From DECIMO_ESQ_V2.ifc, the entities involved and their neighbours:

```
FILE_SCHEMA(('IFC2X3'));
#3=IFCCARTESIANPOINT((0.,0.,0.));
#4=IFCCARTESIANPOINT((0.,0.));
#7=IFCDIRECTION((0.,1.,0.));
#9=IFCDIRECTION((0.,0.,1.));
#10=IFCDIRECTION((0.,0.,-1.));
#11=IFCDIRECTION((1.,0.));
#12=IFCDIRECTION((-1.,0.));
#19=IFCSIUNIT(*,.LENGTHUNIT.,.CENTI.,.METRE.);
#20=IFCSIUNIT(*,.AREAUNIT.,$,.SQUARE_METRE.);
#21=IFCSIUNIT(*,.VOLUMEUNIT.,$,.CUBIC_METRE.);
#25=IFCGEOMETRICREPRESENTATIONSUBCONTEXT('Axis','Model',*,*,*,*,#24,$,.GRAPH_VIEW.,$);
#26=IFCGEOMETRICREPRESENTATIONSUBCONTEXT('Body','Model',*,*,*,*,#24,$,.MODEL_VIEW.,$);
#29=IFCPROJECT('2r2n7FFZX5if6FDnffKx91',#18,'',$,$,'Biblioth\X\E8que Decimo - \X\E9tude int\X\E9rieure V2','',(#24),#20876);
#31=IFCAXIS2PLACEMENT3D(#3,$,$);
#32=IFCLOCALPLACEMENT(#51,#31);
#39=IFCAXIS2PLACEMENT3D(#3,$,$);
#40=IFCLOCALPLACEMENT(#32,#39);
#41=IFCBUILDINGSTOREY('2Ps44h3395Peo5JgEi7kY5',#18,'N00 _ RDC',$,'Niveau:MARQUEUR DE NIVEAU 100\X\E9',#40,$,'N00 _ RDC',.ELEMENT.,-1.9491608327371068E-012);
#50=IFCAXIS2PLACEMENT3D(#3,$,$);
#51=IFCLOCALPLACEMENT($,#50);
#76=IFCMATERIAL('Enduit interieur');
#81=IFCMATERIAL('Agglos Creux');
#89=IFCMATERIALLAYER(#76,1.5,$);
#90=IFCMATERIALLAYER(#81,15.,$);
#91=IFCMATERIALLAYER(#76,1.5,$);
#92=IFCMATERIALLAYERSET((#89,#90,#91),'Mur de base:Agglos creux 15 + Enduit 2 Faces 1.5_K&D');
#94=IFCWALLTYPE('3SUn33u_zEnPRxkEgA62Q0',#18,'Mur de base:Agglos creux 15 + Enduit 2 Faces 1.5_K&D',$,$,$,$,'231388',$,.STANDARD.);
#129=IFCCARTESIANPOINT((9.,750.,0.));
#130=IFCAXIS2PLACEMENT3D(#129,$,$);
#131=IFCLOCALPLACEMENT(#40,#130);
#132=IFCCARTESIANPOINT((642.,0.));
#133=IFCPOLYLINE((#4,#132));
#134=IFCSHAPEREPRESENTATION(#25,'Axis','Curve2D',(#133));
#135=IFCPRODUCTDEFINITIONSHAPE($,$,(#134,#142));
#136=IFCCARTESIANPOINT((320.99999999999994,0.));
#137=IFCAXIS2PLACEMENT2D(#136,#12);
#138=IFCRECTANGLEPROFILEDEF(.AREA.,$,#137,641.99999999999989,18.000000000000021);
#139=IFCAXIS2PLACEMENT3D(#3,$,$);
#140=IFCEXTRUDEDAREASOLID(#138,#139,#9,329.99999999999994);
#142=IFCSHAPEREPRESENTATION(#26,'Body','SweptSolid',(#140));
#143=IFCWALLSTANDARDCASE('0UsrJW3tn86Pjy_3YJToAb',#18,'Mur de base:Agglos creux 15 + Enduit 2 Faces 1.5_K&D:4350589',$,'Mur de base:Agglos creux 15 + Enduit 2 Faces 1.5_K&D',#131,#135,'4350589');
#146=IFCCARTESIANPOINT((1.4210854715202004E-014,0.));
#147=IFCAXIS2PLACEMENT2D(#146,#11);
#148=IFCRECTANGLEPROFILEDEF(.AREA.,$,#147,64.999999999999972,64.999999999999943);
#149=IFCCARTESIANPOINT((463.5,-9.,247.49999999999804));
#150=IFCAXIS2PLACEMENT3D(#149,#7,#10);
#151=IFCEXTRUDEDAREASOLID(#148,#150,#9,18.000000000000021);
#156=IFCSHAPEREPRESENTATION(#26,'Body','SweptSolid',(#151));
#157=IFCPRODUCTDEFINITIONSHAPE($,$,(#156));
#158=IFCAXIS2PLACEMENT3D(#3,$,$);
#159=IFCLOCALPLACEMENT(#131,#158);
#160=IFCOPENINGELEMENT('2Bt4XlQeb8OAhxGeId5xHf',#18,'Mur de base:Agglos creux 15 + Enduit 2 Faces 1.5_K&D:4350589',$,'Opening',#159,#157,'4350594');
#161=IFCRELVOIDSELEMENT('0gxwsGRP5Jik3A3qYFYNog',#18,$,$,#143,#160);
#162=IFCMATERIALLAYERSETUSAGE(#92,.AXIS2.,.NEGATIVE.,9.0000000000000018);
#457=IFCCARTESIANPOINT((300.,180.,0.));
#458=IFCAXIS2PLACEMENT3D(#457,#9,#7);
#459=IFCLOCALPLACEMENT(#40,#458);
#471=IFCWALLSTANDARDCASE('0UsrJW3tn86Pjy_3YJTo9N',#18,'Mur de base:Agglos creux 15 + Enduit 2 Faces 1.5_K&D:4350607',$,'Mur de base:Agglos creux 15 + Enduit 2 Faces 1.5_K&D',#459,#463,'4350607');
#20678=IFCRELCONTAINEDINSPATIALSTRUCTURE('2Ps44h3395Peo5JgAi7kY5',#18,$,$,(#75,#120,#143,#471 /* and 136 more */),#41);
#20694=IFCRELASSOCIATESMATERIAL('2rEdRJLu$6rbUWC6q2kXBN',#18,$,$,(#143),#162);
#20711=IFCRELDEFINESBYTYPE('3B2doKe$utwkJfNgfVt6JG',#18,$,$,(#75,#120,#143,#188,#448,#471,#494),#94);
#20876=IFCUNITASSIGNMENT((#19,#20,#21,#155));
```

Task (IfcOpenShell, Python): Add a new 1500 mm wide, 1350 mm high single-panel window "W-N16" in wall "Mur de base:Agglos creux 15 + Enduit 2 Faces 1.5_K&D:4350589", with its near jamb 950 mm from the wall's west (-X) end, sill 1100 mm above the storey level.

```python
import numpy as np
import ifcopenshell
import ifcopenshell.api.feature
import ifcopenshell.api.geometry
import ifcopenshell.api.root
import ifcopenshell.api.spatial
import ifcopenshell.api.type
import ifcopenshell.geom
import ifcopenshell.util.element
import ifcopenshell.util.placement
import ifcopenshell.util.representation
import ifcopenshell.util.shape
import ifcopenshell.util.unit

model = ifcopenshell.open("DECIMO_ESQ_V2.ifc")
unit_scale = ifcopenshell.util.unit.calculate_unit_scale(model)
settings = ifcopenshell.geom.settings()


def volume(element):
    """Net volume in cubic metres, openings subtracted."""
    shape = ifcopenshell.geom.create_shape(settings, element)
    return ifcopenshell.util.shape.get_volume(shape.geometry)


wall = model.by_guid("0UsrJW3tn86Pjy_3YJToAb")
storey = ifcopenshell.util.element.get_container(wall, ifc_class="IfcBuildingStorey")
context = ifcopenshell.util.representation.get_context(model, "Model", "Body", "MODEL_VIEW")
before = volume(wall)

width, height, from_end, sill = 1.5, 1.35, 0.95, 1.1  # metres

# The wall runs along its own X axis, and the end named is its -X end.
wall_shape = ifcopenshell.geom.create_shape(settings, wall)
x, y, z = ifcopenshell.util.shape.get_vertices(wall_shape.geometry).T
start = x.min() + from_end
face, thickness = float(y.min()), float(y.max() - y.min())
wall_matrix = ifcopenshell.util.placement.get_local_placement(wall.ObjectPlacement)
level = ifcopenshell.util.placement.get_local_placement(storey.ObjectPlacement)[2, 3]


def in_wall(x, y):
    """Placement at x, y metres in the wall's axes, at sill height."""
    matrix = wall_matrix.copy()
    matrix[:, 3] = wall_matrix @ np.array([x / unit_scale, y / unit_scale, 0.0, 1.0])
    matrix[2, 3] = level + sill / unit_scale
    return matrix


# Opening: a box that overshoots both wall faces by 50 mm.
opening = ifcopenshell.api.root.create_entity(model, ifc_class="IfcOpeningElement")
box = ifcopenshell.api.geometry.add_wall_representation(
    model, context=context, length=width, height=height, thickness=thickness + 0.1
)
ifcopenshell.api.geometry.assign_representation(model, product=opening, representation=box)
ifcopenshell.api.geometry.edit_object_placement(model, product=opening, matrix=in_wall(start, face - 0.05), is_si=False)
ifcopenshell.api.feature.add_feature(model, feature=opening, element=wall)

window = ifcopenshell.api.root.create_entity(model, ifc_class="IfcWindow", name="W-N16")
window.OverallWidth, window.OverallHeight = width / unit_scale, height / unit_scale
body = ifcopenshell.api.geometry.add_window_representation(
    model,
    context=context,
    overall_width=window.OverallWidth,
    overall_height=window.OverallHeight,
    partition_type="SINGLE_PANEL",
)
ifcopenshell.api.geometry.assign_representation(model, product=window, representation=body)
ifcopenshell.api.spatial.assign_container(model, products=[window], relating_structure=storey)
fills = ifcopenshell.api.feature.add_filling(model, opening=opening, element=window)
fills.OwnerHistory = window.OwnerHistory  # required in IFC2X3

# IFC2X3 keeps the operation on the window style.
style = ifcopenshell.api.root.create_entity(model, ifc_class="IfcWindowStyle", name="W-N16")
style.OperationType, style.ConstructionType = "SINGLE_PANEL", "NOTDEFINED"
style.ParameterTakesPrecedence = style.Sizeable = False
ifcopenshell.api.type.assign_type(model, related_objects=[window], relating_type=style)

# Centre the window in the wall's thickness.
ifcopenshell.api.geometry.edit_object_placement(model, product=window, matrix=in_wall(start, face), is_si=False)
window_shape = ifcopenshell.geom.create_shape(settings, window)
depth = ifcopenshell.util.shape.get_vertices(window_shape.geometry)[:, 1]
offset = face + thickness / 2 - (depth.min() + depth.max()) / 2
ifcopenshell.api.geometry.edit_object_placement(model, product=window, matrix=in_wall(start, offset), is_si=False)

after = volume(wall)

print(f"wall volume {before:.3f} -> {after:.3f} m3")

model.write("DECIMO_ESQ_V2_updated.ifc")
```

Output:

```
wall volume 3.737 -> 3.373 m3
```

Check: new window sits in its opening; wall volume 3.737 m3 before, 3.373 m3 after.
